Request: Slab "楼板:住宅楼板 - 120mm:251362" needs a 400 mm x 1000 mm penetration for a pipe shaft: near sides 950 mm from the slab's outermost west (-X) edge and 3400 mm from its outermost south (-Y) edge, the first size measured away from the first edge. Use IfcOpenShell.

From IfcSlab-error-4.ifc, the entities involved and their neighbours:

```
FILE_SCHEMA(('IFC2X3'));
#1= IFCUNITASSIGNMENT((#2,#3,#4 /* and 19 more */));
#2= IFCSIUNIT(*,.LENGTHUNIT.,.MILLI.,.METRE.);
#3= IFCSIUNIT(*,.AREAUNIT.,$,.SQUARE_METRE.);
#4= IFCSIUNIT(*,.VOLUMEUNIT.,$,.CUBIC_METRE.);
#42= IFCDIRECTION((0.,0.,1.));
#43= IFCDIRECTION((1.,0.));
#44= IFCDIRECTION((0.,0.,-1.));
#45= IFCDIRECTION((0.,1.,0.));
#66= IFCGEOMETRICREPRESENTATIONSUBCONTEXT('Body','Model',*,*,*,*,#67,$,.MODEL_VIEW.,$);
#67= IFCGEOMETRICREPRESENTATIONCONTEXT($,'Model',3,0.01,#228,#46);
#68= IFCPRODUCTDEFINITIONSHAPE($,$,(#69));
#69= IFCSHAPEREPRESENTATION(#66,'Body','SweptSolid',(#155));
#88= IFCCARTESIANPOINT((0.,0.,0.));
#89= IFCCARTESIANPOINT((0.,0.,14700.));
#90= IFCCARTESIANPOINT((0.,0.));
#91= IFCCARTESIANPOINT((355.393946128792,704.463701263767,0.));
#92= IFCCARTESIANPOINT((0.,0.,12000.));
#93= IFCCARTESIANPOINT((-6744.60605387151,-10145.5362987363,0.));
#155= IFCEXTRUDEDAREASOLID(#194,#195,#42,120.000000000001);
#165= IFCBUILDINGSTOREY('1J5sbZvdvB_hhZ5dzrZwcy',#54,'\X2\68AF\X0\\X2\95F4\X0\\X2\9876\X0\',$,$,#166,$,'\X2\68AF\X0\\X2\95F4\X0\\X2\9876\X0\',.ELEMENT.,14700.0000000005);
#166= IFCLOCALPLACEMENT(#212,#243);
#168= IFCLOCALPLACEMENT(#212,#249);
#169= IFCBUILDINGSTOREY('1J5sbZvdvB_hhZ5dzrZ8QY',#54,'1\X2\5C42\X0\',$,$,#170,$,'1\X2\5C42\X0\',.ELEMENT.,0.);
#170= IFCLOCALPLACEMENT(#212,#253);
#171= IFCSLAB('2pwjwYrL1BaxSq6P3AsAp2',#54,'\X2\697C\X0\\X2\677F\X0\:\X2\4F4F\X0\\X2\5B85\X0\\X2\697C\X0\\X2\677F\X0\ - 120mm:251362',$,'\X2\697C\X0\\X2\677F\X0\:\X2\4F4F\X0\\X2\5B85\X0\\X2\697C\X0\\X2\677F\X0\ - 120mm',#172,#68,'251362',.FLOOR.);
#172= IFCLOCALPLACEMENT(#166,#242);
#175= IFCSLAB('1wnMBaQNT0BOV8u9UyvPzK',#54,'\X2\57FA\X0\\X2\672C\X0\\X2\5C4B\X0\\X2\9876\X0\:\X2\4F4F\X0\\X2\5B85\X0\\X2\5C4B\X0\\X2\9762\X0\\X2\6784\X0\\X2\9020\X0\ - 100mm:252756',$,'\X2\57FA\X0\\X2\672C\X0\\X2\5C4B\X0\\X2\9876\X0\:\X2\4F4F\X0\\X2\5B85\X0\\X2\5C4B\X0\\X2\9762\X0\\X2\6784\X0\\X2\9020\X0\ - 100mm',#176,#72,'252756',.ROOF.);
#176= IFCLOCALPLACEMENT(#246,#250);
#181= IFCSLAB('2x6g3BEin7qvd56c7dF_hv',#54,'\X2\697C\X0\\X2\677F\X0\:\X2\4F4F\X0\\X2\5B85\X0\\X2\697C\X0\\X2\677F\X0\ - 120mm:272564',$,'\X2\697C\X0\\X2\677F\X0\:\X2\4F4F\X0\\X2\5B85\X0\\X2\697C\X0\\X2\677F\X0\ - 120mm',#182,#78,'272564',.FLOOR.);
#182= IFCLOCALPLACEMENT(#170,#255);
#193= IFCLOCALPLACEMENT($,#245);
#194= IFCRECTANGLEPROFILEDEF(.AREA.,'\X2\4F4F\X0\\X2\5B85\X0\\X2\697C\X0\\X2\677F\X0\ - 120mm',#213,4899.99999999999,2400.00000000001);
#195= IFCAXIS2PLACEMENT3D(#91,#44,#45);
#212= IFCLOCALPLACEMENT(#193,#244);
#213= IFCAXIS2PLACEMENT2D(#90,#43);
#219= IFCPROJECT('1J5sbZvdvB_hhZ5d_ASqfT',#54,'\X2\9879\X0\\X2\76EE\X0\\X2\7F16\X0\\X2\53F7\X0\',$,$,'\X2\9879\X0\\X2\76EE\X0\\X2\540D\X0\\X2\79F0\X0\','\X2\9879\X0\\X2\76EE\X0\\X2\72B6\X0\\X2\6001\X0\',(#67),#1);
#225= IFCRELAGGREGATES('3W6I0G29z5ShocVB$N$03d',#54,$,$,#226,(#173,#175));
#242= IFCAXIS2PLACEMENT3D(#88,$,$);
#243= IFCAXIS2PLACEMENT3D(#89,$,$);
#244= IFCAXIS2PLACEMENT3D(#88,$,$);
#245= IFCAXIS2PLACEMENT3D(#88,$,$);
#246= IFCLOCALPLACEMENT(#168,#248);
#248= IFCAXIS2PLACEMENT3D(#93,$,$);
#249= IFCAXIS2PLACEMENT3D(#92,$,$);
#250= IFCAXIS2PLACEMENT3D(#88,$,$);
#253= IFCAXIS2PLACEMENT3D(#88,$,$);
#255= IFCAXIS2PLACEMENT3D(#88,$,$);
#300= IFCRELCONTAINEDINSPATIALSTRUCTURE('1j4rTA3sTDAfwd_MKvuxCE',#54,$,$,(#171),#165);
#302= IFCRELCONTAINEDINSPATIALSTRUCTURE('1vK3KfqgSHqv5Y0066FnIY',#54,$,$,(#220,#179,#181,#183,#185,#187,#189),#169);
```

```python
import numpy as np
import ifcopenshell
import ifcopenshell.api.feature
import ifcopenshell.api.geometry
import ifcopenshell.api.root
import ifcopenshell.geom
import ifcopenshell.util.placement
import ifcopenshell.util.representation
import ifcopenshell.util.shape
import ifcopenshell.util.unit

model = ifcopenshell.open("IfcSlab-error-4.ifc")
unit_scale = ifcopenshell.util.unit.calculate_unit_scale(model)
settings = ifcopenshell.geom.settings()


def volume(element):
    """Net volume in cubic metres, openings subtracted."""
    shape = ifcopenshell.geom.create_shape(settings, element)
    return ifcopenshell.util.shape.get_volume(shape.geometry)


slab = model.by_guid("2pwjwYrL1BaxSq6P3AsAp2")
before = volume(slab)

# Extent in the slab's own axes, in metres. The edges named are its -X and -Y sides.
slab_shape = ifcopenshell.geom.create_shape(settings, slab)
vertices = ifcopenshell.util.shape.get_vertices(slab_shape.geometry)
x_min, y_min, bottom = vertices.min(axis=0)
top = vertices[:, 2].max()

opening = ifcopenshell.api.root.create_entity(model, ifc_class="IfcOpeningElement", name="Pipe shaft opening")
context = ifcopenshell.util.representation.get_context(model, "Model", "Body", "MODEL_VIEW")
width, depth = 0.4, 1
outline = [(0.0, 0.0), (width, 0.0), (width, depth), (0.0, depth), (0.0, 0.0)]
# Overshoot both faces by 50 mm so the cut is clean.
shape = ifcopenshell.api.geometry.add_slab_representation(
    model, context=context, depth=top - bottom + 0.1, polyline=outline
)
ifcopenshell.api.geometry.assign_representation(model, product=opening, representation=shape)

matrix = ifcopenshell.util.placement.get_local_placement(slab.ObjectPlacement)
matrix[:, 3] = matrix @ np.append(np.array([x_min + 0.95, y_min + 3.4, bottom - 0.05]) / unit_scale, 1.0)
ifcopenshell.api.geometry.edit_object_placement(model, product=opening, matrix=matrix, is_si=False)
ifcopenshell.api.feature.add_feature(model, feature=opening, element=slab)

after = volume(slab)

print(f"slab volume {before:.3f} -> {after:.3f} m3")

model.write("IfcSlab-error-4-out.ifc")
```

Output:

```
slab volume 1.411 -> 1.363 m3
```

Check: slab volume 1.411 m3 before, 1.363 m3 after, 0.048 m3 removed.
